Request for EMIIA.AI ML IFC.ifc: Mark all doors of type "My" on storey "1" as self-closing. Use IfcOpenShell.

First a look at what the model holds.

```python
import ifcopenshell
import ifcopenshell.util.element

model = ifcopenshell.open("EMIIA.AI ML IFC.ifc")
print(model.schema)
storey = next(s for s in model.by_type("IfcBuildingStorey") if s.Name == "1")
doors = [e for e in ifcopenshell.util.element.get_decomposition(storey) if e.is_a("IfcDoor")]
seen = {}
for e in doors:
    element_type = ifcopenshell.util.element.get_type(e)
    key = (element_type.Name if element_type != e and element_type else None, ifcopenshell.util.element.get_pset(e, "Pset_DoorCommon", "SelfClosing"))
    seen[key] = seen.get(key, 0) + 1
for (name, value), count in sorted(seen.items(), key=str):
    print(count, "x", name, "|", value)
```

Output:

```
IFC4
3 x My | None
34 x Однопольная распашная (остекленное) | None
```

```python
import ifcopenshell
import ifcopenshell.api.pset
import ifcopenshell.util.element

model = ifcopenshell.open("EMIIA.AI ML IFC.ifc")

storey = next(s for s in model.by_type("IfcBuildingStorey") if s.Name == "1")
doors = [e for e in ifcopenshell.util.element.get_decomposition(storey) if e.is_a("IfcDoor")]

count = 0
for e in doors:
    element_type = ifcopenshell.util.element.get_type(e)
    if element_type in (None, e) or element_type.Name != "My":
        continue
    # add_pset returns the element's existing set when there is one.
    pset = ifcopenshell.api.pset.add_pset(model, product=e, name="Pset_DoorCommon")
    ifcopenshell.api.pset.edit_pset(model, pset=pset, properties={"SelfClosing": True})
    count += 1

print(count, "doors updated")

model.write("EMIIA.AI ML IFC_v2.ifc")
```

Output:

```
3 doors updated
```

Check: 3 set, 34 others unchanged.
